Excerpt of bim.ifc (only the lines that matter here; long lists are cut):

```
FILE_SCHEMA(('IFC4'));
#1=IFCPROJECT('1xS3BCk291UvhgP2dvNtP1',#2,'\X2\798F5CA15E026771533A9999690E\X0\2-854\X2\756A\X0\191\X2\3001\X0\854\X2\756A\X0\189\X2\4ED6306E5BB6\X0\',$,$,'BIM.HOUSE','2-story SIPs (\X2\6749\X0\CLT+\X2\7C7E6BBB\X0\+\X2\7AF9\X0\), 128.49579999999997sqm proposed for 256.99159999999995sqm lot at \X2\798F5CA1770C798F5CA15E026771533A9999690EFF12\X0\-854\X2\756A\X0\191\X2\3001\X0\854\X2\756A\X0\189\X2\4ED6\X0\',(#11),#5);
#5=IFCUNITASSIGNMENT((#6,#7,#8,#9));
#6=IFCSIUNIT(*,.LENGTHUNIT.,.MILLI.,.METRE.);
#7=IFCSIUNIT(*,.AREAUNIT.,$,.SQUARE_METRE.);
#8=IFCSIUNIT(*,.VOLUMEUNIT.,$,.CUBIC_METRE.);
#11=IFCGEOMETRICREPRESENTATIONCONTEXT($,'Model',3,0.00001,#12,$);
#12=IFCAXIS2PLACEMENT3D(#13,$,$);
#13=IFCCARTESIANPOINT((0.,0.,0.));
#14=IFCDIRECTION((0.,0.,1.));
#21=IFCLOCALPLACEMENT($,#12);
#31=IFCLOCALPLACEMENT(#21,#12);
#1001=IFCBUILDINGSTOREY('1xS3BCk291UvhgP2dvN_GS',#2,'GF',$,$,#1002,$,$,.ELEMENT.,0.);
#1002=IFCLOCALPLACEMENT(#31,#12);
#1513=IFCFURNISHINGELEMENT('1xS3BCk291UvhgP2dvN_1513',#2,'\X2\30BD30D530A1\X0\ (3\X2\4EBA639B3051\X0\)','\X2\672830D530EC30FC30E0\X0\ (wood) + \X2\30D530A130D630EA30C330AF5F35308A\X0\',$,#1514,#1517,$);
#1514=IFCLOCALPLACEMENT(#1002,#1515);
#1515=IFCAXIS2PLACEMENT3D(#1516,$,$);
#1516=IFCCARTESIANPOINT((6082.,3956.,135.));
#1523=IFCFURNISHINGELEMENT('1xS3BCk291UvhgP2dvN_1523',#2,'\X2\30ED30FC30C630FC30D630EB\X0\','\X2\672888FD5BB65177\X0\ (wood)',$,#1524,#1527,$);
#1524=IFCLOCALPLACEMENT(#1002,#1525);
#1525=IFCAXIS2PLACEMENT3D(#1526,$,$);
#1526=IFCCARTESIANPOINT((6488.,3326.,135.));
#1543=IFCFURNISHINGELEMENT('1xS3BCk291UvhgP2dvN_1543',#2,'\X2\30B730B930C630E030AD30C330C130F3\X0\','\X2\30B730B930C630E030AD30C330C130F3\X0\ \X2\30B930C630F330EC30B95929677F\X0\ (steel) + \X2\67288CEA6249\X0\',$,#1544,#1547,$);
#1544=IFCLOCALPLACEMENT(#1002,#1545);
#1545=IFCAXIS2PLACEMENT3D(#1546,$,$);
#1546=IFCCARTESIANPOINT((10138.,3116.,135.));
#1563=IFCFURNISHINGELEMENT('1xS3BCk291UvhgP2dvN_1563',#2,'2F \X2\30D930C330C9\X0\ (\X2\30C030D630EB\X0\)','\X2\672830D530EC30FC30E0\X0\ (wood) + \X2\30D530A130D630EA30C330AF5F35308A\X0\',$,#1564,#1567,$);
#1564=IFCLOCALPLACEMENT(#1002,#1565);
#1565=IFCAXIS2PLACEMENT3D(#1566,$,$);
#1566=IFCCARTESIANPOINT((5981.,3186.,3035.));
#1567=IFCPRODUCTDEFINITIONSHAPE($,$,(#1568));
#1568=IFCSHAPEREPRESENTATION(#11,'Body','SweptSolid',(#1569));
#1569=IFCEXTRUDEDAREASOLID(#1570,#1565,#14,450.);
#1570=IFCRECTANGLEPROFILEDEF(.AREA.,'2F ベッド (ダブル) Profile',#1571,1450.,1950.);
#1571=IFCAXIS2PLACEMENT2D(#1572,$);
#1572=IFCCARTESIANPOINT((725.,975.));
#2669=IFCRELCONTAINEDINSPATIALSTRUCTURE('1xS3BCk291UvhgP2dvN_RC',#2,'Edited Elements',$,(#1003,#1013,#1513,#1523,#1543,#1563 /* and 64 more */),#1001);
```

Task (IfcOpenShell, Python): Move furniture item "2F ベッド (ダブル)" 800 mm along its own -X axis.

```python
import ifcopenshell
import ifcopenshell.api.geometry
import ifcopenshell.util.placement

model = ifcopenshell.open("bim.ifc")

item = model.by_guid("1xS3BCk291UvhgP2dvN_1563")
matrix = ifcopenshell.util.placement.get_local_placement(item.ObjectPlacement)
matrix[:3, 3] -= matrix[:3, 0] * 800.0
ifcopenshell.api.geometry.edit_object_placement(model, product=item, matrix=matrix, is_si=False)

print(ifcopenshell.util.placement.get_local_placement(item.ObjectPlacement).round(3) + 0.0)

model.write("bim-out.ifc")
```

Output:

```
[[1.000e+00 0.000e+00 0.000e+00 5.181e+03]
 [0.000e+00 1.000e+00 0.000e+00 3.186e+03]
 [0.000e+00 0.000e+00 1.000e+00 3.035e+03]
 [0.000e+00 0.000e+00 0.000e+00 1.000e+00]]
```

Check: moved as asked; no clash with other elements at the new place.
